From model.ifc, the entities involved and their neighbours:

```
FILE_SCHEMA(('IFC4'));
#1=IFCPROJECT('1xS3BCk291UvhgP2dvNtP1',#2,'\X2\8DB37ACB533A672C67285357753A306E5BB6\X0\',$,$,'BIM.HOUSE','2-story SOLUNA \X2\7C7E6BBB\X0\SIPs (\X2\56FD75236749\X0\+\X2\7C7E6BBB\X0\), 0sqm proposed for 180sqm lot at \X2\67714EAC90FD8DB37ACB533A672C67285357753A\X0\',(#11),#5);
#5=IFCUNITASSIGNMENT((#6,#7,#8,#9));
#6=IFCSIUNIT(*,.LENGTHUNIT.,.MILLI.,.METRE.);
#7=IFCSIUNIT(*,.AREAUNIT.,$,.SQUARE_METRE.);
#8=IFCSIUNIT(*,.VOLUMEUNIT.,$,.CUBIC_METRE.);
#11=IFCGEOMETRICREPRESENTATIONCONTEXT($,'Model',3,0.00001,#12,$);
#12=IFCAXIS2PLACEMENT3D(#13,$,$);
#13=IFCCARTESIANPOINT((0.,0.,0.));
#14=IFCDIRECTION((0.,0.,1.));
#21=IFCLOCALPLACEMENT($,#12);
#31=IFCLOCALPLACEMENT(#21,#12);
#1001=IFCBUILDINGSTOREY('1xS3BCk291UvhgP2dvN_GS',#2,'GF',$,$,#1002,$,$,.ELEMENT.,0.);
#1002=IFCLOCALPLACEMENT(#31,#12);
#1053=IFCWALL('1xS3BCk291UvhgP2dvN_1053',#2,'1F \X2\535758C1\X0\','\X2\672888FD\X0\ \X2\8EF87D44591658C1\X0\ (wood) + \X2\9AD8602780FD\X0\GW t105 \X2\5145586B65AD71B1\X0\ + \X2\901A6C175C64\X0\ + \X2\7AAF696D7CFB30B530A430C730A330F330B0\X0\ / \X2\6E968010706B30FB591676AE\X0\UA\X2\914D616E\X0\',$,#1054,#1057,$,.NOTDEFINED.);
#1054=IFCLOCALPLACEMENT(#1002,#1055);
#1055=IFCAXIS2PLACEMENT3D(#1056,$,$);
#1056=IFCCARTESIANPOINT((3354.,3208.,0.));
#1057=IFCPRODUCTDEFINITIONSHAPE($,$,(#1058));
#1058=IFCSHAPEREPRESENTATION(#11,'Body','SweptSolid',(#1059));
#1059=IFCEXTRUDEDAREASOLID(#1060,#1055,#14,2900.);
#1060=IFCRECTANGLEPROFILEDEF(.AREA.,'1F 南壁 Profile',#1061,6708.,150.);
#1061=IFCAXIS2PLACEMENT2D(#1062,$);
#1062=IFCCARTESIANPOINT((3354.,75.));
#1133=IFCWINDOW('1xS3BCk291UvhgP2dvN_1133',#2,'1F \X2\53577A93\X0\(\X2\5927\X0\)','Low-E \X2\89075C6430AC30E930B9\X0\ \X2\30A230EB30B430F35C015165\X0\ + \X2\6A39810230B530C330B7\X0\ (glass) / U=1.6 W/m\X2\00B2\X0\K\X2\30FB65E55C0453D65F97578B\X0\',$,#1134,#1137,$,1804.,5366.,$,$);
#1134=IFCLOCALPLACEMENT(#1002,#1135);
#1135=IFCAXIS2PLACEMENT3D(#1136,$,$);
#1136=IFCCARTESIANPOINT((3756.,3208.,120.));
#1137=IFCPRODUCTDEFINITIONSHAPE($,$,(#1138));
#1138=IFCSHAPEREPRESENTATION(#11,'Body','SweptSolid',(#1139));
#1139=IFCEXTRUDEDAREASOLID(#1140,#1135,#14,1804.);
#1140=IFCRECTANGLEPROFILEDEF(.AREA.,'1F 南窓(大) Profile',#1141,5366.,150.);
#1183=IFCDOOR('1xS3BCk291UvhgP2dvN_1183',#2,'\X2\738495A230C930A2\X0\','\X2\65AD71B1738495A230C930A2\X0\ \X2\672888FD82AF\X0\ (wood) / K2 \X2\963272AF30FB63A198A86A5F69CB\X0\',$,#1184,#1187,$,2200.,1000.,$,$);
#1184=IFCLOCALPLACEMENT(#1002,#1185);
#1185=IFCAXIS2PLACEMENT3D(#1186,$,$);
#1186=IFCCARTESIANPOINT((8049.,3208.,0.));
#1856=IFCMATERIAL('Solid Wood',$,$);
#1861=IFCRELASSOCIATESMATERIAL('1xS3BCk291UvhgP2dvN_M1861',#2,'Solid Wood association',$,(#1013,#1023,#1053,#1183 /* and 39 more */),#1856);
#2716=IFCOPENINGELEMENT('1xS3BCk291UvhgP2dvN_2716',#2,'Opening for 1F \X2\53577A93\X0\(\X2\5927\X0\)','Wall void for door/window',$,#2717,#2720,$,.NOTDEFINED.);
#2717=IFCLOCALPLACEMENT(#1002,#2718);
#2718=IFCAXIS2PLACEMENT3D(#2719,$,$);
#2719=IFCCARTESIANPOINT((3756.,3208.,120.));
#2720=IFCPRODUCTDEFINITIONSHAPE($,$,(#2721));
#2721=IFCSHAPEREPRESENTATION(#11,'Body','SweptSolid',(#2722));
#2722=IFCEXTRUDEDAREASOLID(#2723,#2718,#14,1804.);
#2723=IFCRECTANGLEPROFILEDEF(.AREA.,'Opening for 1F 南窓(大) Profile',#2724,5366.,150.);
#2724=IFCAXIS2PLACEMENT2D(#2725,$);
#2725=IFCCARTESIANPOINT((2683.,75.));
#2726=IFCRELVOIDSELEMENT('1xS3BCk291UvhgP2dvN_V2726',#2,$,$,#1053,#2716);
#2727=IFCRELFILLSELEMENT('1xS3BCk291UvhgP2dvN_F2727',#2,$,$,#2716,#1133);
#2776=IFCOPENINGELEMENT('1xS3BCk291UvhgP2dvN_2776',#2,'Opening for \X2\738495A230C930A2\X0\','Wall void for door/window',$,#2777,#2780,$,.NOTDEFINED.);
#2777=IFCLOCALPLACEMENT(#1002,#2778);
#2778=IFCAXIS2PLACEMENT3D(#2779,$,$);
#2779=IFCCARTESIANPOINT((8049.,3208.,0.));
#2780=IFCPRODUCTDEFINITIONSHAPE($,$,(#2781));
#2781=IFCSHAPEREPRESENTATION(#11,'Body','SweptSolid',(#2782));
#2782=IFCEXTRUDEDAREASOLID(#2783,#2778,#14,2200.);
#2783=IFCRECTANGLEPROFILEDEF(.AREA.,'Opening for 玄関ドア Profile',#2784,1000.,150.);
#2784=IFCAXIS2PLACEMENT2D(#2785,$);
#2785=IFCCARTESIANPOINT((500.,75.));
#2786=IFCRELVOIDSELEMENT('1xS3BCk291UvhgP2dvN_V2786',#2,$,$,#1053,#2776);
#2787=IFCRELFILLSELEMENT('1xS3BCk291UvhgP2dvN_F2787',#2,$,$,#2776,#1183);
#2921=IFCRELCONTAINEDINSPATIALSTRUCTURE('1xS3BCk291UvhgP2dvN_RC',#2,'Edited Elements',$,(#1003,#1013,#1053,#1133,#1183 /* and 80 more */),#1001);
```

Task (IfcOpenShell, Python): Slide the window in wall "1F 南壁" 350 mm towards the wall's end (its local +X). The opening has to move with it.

```python
import ifcopenshell
import ifcopenshell.api.geometry
import ifcopenshell.util.placement

model = ifcopenshell.open("model.ifc")

window = model.by_guid("1xS3BCk291UvhgP2dvN_1133")
opening = window.FillsVoids[0].RelatingOpeningElement
wall = opening.VoidsElements[0].RelatingBuildingElement

wall_matrix = ifcopenshell.util.placement.get_local_placement(wall.ObjectPlacement)
shift = wall_matrix[:3, 0] * 350.0
before = ifcopenshell.util.placement.get_local_placement(window.ObjectPlacement)[:3, 3].copy()

# The window is not placed relative to its opening, so move both.
for product in (opening, window):
    matrix = ifcopenshell.util.placement.get_local_placement(product.ObjectPlacement)
    matrix[:3, 3] += shift
    ifcopenshell.api.geometry.edit_object_placement(model, product=product, matrix=matrix, is_si=False)

after = ifcopenshell.util.placement.get_local_placement(window.ObjectPlacement)[:3, 3]
print("window moved by", (after - before).round(3) + 0.0)

model.write("model_updated.ifc")
```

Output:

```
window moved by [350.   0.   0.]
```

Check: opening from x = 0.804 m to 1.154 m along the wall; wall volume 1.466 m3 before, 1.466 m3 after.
